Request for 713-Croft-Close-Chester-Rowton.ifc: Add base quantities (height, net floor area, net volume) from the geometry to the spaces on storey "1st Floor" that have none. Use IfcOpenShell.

First a look at what the model holds.

```python
import ifcopenshell
import ifcopenshell.util.element
import ifcopenshell.util.unit

model = ifcopenshell.open("713-Croft-Close-Chester-Rowton.ifc")
print(model.schema)
for unit_type in ("LENGTHUNIT", "AREAUNIT", "VOLUMEUNIT"):
    print(unit_type, ifcopenshell.util.unit.calculate_unit_scale(model, unit_type))
storey = next(s for s in model.by_type("IfcBuildingStorey") if s.Name == "1st Floor")
spaces = [e for e in ifcopenshell.util.element.get_decomposition(storey) if e.is_a("IfcSpace")]
for e in sorted(spaces, key=lambda e: e.id()):
    print(e.id(), e.is_a(), e.Name, list(ifcopenshell.util.element.get_psets(e, qtos_only=True)), sep=" | ")
```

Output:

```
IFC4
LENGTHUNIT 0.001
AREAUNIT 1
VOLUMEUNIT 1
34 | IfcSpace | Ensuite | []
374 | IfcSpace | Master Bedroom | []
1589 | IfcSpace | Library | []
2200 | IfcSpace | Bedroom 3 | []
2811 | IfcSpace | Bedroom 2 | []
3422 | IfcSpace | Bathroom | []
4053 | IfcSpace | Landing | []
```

```python
import ifcopenshell
import ifcopenshell.api.pset
import ifcopenshell.geom
import ifcopenshell.util.element
import ifcopenshell.util.shape
import ifcopenshell.util.unit

model = ifcopenshell.open("713-Croft-Close-Chester-Rowton.ifc")
unit_scale = ifcopenshell.util.unit.calculate_unit_scale(model)
area_scale = ifcopenshell.util.unit.calculate_unit_scale(model, "AREAUNIT")
volume_scale = ifcopenshell.util.unit.calculate_unit_scale(model, "VOLUMEUNIT")
settings = ifcopenshell.geom.settings()

storey = next(s for s in model.by_type("IfcBuildingStorey") if s.Name == "1st Floor")
spaces = [e for e in ifcopenshell.util.element.get_decomposition(storey) if e.is_a("IfcSpace")]

for e in sorted(spaces, key=lambda e: e.id()):
    if ifcopenshell.util.element.get_psets(e, qtos_only=True, should_inherit=False):
        continue
    # Geometry comes back in metres, in the element's own axes.
    shape = ifcopenshell.geom.create_shape(settings, e)
    values = {
        "Height": ifcopenshell.util.shape.get_z(shape.geometry) / unit_scale,
        "NetFloorArea": ifcopenshell.util.shape.get_footprint_area(shape.geometry) / area_scale,
        "NetVolume": ifcopenshell.util.shape.get_volume(shape.geometry) / volume_scale,
    }
    qto = ifcopenshell.api.pset.add_qto(model, product=e, name="Qto_SpaceBaseQuantities")
    ifcopenshell.api.pset.edit_qto(model, qto=qto, properties=values)
    print(e.id(), {k: round(v, 3) for k, v in values.items()})

model.write("713-Croft-Close-Chester-Rowton-out.ifc")
```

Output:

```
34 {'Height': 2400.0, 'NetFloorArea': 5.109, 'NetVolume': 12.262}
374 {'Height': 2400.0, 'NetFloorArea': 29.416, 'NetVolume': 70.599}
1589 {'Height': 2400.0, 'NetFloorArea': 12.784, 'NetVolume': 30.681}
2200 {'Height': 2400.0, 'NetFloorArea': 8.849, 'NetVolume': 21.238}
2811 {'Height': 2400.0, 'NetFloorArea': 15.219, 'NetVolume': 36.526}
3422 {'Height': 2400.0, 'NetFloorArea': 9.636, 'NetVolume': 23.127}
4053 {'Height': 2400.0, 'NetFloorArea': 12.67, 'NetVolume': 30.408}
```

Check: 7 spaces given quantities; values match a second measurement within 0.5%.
